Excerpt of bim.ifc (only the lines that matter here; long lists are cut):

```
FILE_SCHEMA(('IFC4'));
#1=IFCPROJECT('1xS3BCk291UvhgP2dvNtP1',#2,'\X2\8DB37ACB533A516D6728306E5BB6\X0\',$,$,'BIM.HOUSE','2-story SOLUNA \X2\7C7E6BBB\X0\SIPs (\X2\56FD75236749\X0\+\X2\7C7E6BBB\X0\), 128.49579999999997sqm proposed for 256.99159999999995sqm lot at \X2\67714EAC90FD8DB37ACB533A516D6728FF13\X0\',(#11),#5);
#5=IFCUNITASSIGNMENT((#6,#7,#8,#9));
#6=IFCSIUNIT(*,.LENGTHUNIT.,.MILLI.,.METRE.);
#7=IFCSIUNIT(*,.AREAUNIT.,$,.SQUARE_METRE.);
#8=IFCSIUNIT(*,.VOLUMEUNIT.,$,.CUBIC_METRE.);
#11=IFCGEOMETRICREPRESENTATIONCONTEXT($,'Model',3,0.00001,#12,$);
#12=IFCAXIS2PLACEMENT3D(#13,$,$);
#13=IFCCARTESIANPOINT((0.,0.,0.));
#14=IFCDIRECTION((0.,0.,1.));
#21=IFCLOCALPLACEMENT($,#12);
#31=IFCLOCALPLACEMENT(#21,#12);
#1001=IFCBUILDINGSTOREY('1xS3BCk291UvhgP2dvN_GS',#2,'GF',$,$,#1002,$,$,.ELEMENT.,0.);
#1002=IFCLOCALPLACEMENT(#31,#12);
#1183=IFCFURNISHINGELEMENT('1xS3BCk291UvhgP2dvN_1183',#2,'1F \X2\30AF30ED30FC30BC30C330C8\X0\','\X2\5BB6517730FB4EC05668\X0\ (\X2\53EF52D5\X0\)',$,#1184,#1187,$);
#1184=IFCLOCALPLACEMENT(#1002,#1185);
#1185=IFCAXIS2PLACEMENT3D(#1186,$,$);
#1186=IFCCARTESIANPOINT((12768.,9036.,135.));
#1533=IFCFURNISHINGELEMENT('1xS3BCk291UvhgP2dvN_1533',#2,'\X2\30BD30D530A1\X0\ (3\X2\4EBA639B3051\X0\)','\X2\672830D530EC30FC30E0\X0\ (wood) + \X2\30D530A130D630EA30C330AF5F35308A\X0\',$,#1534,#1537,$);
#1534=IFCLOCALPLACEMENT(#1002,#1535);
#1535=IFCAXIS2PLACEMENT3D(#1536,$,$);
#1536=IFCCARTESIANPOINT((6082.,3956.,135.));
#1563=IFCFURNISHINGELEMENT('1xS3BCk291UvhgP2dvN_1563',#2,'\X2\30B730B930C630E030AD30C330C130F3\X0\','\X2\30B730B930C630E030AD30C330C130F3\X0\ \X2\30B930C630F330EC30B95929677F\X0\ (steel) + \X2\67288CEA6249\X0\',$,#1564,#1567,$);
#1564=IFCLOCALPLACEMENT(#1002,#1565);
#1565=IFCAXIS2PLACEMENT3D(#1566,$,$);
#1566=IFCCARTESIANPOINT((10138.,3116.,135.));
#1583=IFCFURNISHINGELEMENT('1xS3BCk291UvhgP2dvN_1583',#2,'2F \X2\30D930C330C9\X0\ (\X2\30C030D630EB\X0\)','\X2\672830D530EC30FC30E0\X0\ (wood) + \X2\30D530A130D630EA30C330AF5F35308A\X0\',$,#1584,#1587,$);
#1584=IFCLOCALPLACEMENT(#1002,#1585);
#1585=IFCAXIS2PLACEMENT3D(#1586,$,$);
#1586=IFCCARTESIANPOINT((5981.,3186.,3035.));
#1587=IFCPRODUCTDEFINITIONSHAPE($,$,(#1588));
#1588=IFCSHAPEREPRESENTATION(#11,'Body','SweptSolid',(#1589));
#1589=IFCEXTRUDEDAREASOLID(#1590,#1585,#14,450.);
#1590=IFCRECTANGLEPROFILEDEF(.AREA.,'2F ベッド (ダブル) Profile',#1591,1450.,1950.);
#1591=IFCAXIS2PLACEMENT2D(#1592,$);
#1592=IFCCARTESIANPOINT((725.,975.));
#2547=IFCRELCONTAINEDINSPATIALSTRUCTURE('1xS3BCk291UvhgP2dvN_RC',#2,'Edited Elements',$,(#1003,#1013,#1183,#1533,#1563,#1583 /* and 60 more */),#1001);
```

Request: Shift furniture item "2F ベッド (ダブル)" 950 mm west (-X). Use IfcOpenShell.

```python
import ifcopenshell
import ifcopenshell.api.geometry
import ifcopenshell.util.placement

model = ifcopenshell.open("bim.ifc")

item = model.by_id(1583)
matrix = ifcopenshell.util.placement.get_local_placement(item.ObjectPlacement)
matrix[0, 3] -= 950.0
ifcopenshell.api.geometry.edit_object_placement(model, product=item, matrix=matrix, is_si=False)

print(ifcopenshell.util.placement.get_local_placement(item.ObjectPlacement).round(3) + 0.0)

model.write("bim_edited.ifc")
```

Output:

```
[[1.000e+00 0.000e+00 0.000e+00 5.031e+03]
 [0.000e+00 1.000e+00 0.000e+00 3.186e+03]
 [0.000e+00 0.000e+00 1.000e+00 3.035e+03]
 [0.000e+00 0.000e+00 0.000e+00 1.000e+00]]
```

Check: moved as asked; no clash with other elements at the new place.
